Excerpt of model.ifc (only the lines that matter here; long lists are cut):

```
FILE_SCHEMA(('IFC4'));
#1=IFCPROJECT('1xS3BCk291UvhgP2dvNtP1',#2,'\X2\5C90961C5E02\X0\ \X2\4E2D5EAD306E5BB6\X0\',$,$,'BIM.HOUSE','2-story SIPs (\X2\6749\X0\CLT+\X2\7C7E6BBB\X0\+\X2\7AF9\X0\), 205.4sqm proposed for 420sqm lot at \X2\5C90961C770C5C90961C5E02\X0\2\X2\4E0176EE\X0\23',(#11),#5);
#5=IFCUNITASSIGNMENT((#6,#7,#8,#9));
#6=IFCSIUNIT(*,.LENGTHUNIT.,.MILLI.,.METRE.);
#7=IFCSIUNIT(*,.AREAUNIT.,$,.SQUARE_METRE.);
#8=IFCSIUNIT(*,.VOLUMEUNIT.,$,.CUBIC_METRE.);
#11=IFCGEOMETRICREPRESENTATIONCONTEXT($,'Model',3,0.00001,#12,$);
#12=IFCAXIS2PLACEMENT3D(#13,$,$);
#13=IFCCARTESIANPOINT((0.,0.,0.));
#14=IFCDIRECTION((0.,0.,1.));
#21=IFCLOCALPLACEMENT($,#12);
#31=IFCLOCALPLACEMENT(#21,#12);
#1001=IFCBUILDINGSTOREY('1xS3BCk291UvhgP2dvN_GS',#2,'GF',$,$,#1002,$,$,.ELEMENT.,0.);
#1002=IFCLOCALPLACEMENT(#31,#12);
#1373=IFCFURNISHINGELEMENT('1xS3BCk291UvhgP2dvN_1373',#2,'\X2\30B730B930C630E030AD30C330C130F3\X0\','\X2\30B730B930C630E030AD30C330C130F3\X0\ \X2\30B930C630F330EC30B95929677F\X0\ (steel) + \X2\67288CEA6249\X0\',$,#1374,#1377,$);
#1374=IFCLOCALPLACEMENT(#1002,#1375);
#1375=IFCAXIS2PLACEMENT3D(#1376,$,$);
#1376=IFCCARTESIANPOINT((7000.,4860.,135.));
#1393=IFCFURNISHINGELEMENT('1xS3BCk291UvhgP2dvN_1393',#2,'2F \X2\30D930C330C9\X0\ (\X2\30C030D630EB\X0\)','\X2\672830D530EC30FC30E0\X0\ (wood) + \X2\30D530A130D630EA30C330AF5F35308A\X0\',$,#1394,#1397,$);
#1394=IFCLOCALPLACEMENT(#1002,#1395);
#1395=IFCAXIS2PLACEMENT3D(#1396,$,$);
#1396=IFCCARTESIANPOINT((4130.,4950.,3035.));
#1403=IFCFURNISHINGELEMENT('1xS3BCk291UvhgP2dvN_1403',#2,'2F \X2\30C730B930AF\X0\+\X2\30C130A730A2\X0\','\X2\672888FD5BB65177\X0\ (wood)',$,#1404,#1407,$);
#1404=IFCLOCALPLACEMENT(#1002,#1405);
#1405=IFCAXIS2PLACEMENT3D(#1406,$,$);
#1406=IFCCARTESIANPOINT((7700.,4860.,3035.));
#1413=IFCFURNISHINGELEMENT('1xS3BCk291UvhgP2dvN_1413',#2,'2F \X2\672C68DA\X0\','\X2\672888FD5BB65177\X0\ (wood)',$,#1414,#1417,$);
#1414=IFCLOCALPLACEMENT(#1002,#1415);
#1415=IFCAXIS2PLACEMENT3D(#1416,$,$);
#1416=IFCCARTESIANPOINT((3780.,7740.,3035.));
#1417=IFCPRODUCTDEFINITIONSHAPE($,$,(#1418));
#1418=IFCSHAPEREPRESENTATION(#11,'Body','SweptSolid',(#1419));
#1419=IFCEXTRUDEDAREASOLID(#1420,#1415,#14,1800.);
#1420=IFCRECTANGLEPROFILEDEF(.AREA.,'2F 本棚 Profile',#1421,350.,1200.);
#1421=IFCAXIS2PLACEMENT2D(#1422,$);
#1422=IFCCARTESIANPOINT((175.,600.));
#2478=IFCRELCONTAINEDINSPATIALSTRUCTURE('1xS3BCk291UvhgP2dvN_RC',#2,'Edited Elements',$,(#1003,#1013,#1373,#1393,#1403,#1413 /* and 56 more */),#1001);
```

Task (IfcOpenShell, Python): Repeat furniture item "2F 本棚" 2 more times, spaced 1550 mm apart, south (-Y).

```python
import numpy as np
import ifcopenshell
import ifcopenshell.api.geometry
import ifcopenshell.api.root
import ifcopenshell.util.element
import ifcopenshell.util.placement
import ifcopenshell.util.unit

model = ifcopenshell.open("model.ifc")
unit_scale = ifcopenshell.util.unit.calculate_unit_scale(model)


def reuse_history(source, copy):
    """copy_class also copies each property set's owner history, people and application; keep the originals."""
    for rel in copy.IsDefinedBy:
        if rel.is_a("IfcRelDefinesByProperties") and (history := rel.RelatingPropertyDefinition.OwnerHistory):
            rel.RelatingPropertyDefinition.OwnerHistory = source.OwnerHistory
            ifcopenshell.util.element.remove_deep2(model, history)


source = model.by_guid("1xS3BCk291UvhgP2dvN_1413")
base = ifcopenshell.util.placement.get_local_placement(source.ObjectPlacement)
step = np.array([0.0, -1.0, 0.0]) * 1.55 / unit_scale

for i in range(1, 3):
    copy = ifcopenshell.api.root.copy_class(model, product=source)
    copy.Representation = ifcopenshell.util.element.copy_deep(
        model, source.Representation, exclude=["IfcGeometricRepresentationContext", "IfcRepresentationMap"]
    )
    reuse_history(source, copy)
    matrix = base.copy()
    matrix[:3, 3] += i * step
    print("added at", matrix[:3, 3].round(3) + 0.0)
    ifcopenshell.api.geometry.edit_object_placement(model, product=copy, matrix=matrix, is_si=False)

model.write("model-out.ifc")
```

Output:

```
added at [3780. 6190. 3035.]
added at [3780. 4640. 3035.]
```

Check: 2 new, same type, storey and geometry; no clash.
